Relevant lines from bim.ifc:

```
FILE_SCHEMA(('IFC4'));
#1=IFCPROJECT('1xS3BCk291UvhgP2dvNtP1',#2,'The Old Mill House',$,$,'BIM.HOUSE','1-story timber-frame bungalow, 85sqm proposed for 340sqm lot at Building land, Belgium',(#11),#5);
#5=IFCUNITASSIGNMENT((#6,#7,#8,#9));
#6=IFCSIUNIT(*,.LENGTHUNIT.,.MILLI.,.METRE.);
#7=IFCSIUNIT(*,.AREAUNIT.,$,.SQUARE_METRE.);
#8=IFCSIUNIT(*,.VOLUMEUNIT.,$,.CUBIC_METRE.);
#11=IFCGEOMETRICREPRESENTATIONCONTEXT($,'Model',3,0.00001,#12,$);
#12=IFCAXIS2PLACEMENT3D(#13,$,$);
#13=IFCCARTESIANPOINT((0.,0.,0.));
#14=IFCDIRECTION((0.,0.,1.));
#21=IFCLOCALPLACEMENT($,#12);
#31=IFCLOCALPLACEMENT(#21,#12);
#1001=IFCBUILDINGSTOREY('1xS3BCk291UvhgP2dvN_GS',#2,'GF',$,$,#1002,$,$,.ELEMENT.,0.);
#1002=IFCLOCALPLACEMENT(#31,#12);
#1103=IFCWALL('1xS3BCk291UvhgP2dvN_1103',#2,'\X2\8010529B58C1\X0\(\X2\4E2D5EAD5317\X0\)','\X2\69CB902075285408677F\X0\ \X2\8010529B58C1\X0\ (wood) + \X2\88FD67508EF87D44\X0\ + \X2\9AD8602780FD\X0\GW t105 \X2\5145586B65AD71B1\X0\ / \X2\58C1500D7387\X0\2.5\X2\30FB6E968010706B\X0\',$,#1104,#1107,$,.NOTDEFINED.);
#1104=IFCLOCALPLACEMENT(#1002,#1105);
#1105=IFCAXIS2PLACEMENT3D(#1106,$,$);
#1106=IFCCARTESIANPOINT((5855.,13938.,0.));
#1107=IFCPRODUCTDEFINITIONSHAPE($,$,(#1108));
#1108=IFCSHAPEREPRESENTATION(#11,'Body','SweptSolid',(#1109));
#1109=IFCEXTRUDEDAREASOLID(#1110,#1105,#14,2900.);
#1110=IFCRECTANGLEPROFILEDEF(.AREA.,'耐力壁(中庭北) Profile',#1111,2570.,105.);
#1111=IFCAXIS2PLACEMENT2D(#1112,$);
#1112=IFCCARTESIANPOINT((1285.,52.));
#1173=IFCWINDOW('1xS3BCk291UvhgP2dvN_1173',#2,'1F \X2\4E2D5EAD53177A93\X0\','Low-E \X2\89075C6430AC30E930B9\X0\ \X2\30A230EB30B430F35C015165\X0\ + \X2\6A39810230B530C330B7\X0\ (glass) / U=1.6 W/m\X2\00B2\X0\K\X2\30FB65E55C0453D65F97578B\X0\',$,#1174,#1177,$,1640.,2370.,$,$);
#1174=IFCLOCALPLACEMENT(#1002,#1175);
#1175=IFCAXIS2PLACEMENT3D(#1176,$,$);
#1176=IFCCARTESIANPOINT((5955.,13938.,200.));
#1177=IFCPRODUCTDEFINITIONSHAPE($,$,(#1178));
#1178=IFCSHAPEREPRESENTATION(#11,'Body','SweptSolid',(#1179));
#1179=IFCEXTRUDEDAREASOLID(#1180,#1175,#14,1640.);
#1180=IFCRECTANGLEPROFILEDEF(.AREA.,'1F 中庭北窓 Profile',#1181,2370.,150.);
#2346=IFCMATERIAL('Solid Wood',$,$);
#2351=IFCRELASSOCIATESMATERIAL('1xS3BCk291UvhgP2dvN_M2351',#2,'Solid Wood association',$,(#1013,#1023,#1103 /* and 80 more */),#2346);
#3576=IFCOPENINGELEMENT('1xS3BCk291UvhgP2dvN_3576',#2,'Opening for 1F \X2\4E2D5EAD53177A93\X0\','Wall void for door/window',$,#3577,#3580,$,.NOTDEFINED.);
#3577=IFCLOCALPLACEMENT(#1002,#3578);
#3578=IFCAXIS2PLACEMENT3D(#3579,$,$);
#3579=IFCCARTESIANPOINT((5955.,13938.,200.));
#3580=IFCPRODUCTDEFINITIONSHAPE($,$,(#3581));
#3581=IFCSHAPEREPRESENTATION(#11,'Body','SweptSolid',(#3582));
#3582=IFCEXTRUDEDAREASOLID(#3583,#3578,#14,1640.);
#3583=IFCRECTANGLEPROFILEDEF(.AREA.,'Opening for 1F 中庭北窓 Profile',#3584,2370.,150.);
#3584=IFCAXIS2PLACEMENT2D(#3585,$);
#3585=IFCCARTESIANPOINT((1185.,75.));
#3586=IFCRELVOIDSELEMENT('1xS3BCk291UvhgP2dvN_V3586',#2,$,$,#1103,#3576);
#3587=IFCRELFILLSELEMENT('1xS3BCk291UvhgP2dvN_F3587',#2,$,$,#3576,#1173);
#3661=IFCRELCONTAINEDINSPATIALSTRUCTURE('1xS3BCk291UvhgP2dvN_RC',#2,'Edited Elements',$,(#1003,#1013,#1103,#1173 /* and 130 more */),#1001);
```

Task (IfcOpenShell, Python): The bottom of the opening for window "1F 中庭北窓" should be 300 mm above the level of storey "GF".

```python
import numpy as np
import ifcopenshell
import ifcopenshell.api.geometry
import ifcopenshell.geom
import ifcopenshell.util.element
import ifcopenshell.util.placement
import ifcopenshell.util.shape
import ifcopenshell.util.unit

model = ifcopenshell.open("bim.ifc")
unit_scale = ifcopenshell.util.unit.calculate_unit_scale(model)

window = model.by_guid("1xS3BCk291UvhgP2dvN_1173")
opening = window.FillsVoids[0].RelatingOpeningElement
storey = ifcopenshell.util.element.get_container(window, ifc_class="IfcBuildingStorey")
level = ifcopenshell.util.placement.get_local_placement(storey.ObjectPlacement)[2, 3]

# The opening's origin need not be at the sill, so measure its lowest point.
shape = ifcopenshell.geom.create_shape(ifcopenshell.geom.settings(), opening)
bottom = ifcopenshell.util.shape.get_shape_bottom_elevation(shape, shape.geometry) / unit_scale
dz = level + 0.3 / unit_scale - bottom

shift = np.array([0.0, 0.0, dz])
# The window is not placed relative to its opening, so move both.
for product in (opening, window):
    matrix = ifcopenshell.util.placement.get_local_placement(product.ObjectPlacement)
    matrix[:3, 3] += shift
    ifcopenshell.api.geometry.edit_object_placement(model, product=product, matrix=matrix, is_si=False)

print(f"moved by {dz * unit_scale:+.3f} m")

model.write("bim-out.ifc")
```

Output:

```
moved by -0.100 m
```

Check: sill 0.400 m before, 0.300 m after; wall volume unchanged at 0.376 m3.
